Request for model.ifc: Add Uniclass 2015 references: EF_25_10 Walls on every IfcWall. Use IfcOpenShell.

First a look at what the model holds.

```python
import ifcopenshell

model = ifcopenshell.open("model.ifc")
print(model.schema)
print("classifications:", [c.Name for c in model.by_type("IfcClassification")])
for ifc_class in ("IfcDoor", "IfcRoof", "IfcStair", "IfcWall", "IfcWindow"):
    print(ifc_class, len(model.by_type(ifc_class)))
```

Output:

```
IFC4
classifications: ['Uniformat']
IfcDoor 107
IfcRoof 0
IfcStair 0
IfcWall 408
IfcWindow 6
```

```python
import ifcopenshell
import ifcopenshell.api.classification

model = ifcopenshell.open("model.ifc")

system = ifcopenshell.api.classification.add_classification(model, classification="Uniclass 2015")

codes = {
    "IfcWall": ("EF_25_10", "Walls"),
}
for ifc_class, (code, name) in codes.items():
    products = model.by_type(ifc_class)
    ifcopenshell.api.classification.add_reference(
        model, products=products, classification=system, identification=code, name=name
    )
    print(code, len(products))

model.write("model_edited.ifc")
```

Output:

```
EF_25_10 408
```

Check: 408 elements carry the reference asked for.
